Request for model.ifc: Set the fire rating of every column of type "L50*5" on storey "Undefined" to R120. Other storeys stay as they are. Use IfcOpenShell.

First a look at what the model holds.

```python
import ifcopenshell
import ifcopenshell.util.element

model = ifcopenshell.open("model.ifc")
print(model.schema)
storey = next(s for s in model.by_type("IfcBuildingStorey") if s.Name == "Undefined")
columns = [e for e in ifcopenshell.util.element.get_decomposition(storey) if e.is_a("IfcColumn")]
seen = {}
for e in columns:
    element_type = ifcopenshell.util.element.get_type(e)
    key = (element_type.Name if element_type != e and element_type else None, ifcopenshell.util.element.get_pset(e, "Pset_ColumnCommon", "FireRating"))
    seen[key] = seen.get(key, 0) + 1
for (name, value), count in sorted(seen.items(), key=str):
    print(count, "x", name, "|", value)
```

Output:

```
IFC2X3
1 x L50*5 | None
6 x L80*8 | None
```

```python
import ifcopenshell
import ifcopenshell.api.pset
import ifcopenshell.util.element

model = ifcopenshell.open("model.ifc")

storey = next(s for s in model.by_type("IfcBuildingStorey") if s.Name == "Undefined")
columns = [e for e in ifcopenshell.util.element.get_decomposition(storey) if e.is_a("IfcColumn")]

count = 0
for e in columns:
    element_type = ifcopenshell.util.element.get_type(e)
    if element_type in (None, e) or element_type.Name != "L50*5":
        continue
    # add_pset returns the element's existing set when there is one.
    pset = ifcopenshell.api.pset.add_pset(model, product=e, name="Pset_ColumnCommon")
    ifcopenshell.api.pset.edit_pset(model, pset=pset, properties={"FireRating": "R120"})
    count += 1

print(count, "columns updated")

model.write("model-out.ifc")
```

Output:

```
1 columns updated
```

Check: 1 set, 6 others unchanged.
